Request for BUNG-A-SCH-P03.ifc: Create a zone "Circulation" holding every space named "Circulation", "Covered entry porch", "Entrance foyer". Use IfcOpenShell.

First a look at what the model holds.

```python
import ifcopenshell

model = ifcopenshell.open("BUNG-A-SCH-P03.ifc")
print(model.schema)
seen = {}
for space in model.by_type("IfcSpace"):
    seen[space.LongName] = seen.get(space.LongName, 0) + 1
for name, count in sorted(seen.items(), key=str):
    print(count, "x", name)
print("zones:", [z.Name for z in model.by_type("IfcZone")][:20])
```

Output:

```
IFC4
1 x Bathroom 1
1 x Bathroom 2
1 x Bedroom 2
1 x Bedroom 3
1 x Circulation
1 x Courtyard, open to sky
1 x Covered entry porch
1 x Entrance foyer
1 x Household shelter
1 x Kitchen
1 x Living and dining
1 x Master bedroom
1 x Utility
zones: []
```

```python
import ifcopenshell
import ifcopenshell.api.group
import ifcopenshell.api.root

model = ifcopenshell.open("BUNG-A-SCH-P03.ifc")

names = {"Circulation", "Covered entry porch", "Entrance foyer"}
spaces = [s for s in model.by_type("IfcSpace") if s.LongName in names]

zone = ifcopenshell.api.root.create_entity(model, ifc_class="IfcZone", name="Circulation")
ifcopenshell.api.group.assign_group(model, products=spaces, group=zone)
print(len(spaces), "spaces in", zone.Name)

model.write("BUNG-A-SCH-P03_updated.ifc")
```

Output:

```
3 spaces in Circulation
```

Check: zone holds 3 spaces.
